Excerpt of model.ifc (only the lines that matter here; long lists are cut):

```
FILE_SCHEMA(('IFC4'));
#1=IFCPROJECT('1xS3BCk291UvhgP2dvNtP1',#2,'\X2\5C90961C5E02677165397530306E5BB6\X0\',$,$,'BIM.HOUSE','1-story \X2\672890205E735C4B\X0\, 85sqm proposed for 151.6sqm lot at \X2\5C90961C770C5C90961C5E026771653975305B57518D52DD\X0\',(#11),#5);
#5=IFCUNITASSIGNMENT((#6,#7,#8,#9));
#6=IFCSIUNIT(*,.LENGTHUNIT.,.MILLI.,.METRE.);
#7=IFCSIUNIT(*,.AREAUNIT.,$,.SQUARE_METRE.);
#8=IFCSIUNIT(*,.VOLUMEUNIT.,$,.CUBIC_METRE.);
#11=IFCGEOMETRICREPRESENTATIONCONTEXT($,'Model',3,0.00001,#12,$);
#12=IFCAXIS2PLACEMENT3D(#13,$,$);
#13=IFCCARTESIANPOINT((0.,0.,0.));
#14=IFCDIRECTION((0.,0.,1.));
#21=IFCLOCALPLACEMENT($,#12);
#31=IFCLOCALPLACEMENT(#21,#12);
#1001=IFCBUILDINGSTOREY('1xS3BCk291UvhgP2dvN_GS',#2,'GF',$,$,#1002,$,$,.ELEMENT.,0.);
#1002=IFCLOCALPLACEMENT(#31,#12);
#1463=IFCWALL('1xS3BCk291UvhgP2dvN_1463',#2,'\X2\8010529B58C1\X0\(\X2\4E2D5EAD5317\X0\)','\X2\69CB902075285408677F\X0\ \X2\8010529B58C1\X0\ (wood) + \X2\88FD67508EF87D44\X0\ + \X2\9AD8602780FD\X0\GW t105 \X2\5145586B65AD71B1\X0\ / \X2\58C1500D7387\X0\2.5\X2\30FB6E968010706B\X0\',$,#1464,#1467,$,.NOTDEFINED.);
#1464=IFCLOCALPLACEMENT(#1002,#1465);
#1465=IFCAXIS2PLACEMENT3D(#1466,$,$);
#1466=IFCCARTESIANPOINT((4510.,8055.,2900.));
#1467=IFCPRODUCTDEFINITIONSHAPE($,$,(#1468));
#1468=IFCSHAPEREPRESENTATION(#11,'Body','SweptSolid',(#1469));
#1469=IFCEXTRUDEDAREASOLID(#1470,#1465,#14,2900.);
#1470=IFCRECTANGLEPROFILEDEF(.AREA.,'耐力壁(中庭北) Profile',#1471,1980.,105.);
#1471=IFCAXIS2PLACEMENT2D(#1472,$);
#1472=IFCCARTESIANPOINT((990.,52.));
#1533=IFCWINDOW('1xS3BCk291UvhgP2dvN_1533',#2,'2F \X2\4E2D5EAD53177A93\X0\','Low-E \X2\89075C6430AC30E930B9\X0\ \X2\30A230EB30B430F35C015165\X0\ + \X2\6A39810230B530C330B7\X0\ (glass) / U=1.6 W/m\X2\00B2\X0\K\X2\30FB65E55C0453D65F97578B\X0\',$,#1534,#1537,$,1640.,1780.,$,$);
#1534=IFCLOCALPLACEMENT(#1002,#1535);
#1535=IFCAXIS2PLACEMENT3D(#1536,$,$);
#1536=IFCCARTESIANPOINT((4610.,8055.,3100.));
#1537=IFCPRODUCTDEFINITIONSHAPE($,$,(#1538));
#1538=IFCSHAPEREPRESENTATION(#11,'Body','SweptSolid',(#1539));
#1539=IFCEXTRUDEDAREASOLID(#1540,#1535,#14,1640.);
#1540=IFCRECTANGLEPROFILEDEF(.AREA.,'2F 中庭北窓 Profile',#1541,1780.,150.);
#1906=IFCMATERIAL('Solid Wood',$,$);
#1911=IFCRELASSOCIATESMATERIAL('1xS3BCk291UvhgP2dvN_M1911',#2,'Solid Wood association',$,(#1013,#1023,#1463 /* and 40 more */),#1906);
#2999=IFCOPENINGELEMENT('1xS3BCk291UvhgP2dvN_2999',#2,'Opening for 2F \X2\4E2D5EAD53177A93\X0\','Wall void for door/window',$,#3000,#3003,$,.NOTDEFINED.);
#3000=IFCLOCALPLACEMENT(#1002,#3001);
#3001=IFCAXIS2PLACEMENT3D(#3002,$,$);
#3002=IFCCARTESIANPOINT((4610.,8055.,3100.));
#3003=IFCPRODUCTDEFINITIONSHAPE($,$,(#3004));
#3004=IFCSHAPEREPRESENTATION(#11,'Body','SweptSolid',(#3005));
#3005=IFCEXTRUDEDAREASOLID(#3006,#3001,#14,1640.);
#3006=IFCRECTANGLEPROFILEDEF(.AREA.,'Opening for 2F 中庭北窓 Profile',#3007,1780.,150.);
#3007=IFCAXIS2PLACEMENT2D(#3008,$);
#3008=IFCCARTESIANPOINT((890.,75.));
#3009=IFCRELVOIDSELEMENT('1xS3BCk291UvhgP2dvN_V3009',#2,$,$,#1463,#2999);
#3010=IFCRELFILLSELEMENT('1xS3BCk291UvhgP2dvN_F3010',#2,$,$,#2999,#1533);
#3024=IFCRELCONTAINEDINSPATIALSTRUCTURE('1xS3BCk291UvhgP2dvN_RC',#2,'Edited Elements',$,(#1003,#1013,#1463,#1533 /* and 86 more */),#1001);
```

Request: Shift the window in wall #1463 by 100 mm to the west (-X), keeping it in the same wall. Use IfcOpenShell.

```python
import ifcopenshell
import ifcopenshell.api.geometry
import ifcopenshell.util.placement

model = ifcopenshell.open("model.ifc")

window = model.by_id(1533)
opening = window.FillsVoids[0].RelatingOpeningElement
wall = opening.VoidsElements[0].RelatingBuildingElement

wall_matrix = ifcopenshell.util.placement.get_local_placement(wall.ObjectPlacement)
shift = wall_matrix[:3, 0] * -100.0
before = ifcopenshell.util.placement.get_local_placement(window.ObjectPlacement)[:3, 3].copy()

# The window is not placed relative to its opening, so move both.
for product in (opening, window):
    matrix = ifcopenshell.util.placement.get_local_placement(product.ObjectPlacement)
    matrix[:3, 3] += shift
    ifcopenshell.api.geometry.edit_object_placement(model, product=product, matrix=matrix, is_si=False)

after = ifcopenshell.util.placement.get_local_placement(window.ObjectPlacement)[:3, 3]
print("window moved by", (after - before).round(3) + 0.0)

model.write("model_v2.ifc")
```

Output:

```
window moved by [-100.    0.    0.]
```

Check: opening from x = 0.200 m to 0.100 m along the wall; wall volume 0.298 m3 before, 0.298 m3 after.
